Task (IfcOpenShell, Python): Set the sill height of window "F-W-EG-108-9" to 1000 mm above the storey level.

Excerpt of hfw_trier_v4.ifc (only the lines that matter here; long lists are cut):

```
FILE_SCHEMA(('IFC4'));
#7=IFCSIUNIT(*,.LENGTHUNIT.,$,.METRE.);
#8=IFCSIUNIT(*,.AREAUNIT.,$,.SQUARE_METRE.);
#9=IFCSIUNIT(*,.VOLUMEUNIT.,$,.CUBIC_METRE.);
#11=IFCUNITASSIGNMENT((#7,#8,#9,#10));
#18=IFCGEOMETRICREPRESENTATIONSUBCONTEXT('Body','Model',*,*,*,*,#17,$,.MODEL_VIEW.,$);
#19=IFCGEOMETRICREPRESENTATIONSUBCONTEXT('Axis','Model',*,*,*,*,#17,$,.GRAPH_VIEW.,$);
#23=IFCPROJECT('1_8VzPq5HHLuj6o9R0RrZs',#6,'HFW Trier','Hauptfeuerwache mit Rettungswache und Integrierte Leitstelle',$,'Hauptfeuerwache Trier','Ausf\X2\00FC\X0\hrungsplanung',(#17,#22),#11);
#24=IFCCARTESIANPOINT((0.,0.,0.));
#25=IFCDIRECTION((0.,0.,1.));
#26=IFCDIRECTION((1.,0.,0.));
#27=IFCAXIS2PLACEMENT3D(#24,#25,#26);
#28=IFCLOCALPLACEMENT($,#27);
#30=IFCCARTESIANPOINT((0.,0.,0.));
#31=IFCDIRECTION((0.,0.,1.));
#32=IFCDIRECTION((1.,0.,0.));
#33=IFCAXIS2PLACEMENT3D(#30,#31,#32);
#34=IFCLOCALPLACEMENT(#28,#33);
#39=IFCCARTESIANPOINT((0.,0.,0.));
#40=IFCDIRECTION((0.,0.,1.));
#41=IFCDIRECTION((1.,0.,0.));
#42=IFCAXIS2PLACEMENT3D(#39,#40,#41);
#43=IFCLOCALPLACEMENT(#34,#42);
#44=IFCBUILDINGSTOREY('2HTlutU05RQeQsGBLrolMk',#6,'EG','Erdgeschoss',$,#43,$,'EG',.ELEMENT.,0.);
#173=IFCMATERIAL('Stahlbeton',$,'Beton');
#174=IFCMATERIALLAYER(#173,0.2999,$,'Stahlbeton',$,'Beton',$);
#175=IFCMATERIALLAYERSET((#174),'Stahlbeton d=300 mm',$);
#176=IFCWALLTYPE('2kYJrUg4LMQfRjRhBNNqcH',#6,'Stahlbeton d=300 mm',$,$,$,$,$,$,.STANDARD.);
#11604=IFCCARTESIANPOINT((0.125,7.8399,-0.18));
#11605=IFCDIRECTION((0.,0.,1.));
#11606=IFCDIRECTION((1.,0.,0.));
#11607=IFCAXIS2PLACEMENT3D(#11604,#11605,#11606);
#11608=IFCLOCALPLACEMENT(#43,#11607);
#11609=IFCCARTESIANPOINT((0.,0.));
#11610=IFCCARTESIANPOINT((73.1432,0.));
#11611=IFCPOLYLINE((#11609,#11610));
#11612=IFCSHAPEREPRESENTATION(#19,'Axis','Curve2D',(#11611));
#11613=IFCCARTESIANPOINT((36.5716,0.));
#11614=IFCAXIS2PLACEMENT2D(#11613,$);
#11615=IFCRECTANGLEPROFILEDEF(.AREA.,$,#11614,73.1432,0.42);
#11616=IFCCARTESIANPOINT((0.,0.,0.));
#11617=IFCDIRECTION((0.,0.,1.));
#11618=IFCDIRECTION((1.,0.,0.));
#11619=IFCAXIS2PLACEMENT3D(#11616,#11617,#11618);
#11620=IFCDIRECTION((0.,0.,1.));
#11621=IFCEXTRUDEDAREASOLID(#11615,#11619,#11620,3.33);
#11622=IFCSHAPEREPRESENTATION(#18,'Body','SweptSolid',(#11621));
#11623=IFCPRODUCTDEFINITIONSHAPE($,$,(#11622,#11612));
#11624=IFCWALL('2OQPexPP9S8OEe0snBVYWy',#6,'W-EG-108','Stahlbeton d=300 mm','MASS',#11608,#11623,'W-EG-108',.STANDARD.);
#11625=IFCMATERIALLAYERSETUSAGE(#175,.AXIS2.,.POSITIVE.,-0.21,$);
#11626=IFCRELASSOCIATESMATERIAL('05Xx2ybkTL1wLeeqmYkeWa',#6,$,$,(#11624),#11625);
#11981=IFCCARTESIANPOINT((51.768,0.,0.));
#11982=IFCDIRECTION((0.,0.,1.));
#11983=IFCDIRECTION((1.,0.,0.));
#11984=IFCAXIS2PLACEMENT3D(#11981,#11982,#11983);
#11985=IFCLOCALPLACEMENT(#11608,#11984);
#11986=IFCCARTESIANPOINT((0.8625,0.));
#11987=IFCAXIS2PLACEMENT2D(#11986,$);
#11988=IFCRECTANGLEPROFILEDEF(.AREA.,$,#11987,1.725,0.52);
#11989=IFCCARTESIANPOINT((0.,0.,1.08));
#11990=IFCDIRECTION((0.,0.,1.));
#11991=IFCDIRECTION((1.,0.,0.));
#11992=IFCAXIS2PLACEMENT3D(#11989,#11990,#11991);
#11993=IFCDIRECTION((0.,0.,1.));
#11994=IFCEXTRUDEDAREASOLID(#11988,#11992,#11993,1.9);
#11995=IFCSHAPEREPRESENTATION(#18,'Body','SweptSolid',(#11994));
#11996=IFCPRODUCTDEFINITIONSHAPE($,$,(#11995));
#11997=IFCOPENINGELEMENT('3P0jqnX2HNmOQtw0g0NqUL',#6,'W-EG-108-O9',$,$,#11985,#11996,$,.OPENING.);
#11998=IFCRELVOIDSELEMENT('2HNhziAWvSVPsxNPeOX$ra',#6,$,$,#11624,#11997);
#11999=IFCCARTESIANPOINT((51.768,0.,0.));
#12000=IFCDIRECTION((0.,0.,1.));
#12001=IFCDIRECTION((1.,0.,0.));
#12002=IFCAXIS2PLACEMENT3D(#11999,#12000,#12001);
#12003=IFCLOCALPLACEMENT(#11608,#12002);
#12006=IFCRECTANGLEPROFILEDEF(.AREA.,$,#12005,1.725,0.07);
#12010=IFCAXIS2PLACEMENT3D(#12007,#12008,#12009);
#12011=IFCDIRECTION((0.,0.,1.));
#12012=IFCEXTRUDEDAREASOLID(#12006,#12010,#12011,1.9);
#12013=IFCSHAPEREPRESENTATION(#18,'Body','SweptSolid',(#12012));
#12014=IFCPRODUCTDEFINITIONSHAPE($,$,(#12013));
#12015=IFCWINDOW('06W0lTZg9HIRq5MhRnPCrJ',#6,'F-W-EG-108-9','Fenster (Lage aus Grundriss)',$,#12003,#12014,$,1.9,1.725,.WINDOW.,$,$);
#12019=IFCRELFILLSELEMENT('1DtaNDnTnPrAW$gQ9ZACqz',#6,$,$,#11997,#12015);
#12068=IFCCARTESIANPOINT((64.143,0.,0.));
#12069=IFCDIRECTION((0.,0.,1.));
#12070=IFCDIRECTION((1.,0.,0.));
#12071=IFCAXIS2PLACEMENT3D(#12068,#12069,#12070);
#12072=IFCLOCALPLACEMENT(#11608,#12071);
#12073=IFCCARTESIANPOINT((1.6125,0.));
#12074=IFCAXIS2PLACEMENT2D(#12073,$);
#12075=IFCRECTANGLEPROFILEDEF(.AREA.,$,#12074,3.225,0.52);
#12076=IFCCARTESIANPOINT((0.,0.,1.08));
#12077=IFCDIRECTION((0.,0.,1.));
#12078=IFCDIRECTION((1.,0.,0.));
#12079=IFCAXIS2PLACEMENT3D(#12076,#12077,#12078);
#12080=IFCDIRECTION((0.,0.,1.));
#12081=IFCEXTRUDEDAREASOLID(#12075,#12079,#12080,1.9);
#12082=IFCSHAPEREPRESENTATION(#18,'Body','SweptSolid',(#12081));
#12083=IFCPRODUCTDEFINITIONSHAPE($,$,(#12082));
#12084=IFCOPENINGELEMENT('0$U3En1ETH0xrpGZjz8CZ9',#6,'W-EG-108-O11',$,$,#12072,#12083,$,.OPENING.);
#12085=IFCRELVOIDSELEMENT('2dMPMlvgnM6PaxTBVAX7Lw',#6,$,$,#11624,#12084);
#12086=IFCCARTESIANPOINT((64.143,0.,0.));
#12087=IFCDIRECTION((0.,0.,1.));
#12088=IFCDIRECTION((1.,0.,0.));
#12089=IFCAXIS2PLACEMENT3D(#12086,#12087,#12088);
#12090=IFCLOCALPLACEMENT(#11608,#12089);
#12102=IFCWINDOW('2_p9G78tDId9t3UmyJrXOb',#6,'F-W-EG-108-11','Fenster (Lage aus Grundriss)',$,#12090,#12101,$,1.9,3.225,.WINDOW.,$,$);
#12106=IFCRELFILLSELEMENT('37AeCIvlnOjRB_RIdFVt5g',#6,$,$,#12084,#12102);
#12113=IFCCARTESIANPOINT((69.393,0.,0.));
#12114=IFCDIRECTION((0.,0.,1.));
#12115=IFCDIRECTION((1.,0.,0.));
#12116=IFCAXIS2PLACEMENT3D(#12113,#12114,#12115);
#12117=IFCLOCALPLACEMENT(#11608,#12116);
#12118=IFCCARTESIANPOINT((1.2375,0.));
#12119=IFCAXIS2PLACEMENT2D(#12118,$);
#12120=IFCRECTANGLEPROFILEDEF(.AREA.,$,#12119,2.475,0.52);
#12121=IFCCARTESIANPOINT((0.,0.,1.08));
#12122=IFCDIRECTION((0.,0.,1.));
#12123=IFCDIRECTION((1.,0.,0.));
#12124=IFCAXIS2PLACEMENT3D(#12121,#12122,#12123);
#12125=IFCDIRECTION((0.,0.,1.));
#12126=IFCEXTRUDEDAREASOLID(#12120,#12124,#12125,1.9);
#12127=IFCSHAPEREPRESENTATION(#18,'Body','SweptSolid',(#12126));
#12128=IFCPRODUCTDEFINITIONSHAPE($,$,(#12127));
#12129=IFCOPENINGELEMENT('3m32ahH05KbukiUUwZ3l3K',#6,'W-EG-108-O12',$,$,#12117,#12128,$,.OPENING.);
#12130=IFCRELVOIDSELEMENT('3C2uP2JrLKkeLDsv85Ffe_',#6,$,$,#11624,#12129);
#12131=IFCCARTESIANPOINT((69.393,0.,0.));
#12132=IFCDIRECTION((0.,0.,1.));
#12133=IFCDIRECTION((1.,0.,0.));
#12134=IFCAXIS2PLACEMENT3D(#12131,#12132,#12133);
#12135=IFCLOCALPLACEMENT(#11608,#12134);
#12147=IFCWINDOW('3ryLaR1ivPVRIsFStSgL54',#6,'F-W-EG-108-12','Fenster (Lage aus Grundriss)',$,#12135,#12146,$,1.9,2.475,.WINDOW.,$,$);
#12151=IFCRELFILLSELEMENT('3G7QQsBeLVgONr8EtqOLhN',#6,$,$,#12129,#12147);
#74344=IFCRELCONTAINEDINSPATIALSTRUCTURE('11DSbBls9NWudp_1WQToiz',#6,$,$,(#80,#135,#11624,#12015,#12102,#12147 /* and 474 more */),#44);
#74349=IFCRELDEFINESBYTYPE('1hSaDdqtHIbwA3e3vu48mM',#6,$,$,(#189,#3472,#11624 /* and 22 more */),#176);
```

```python
import numpy as np
import ifcopenshell
import ifcopenshell.api.geometry
import ifcopenshell.geom
import ifcopenshell.util.element
import ifcopenshell.util.placement
import ifcopenshell.util.shape
import ifcopenshell.util.unit

model = ifcopenshell.open("hfw_trier_v4.ifc")
unit_scale = ifcopenshell.util.unit.calculate_unit_scale(model)

window = model.by_guid("06W0lTZg9HIRq5MhRnPCrJ")
opening = window.FillsVoids[0].RelatingOpeningElement
storey = ifcopenshell.util.element.get_container(window, ifc_class="IfcBuildingStorey")
level = ifcopenshell.util.placement.get_local_placement(storey.ObjectPlacement)[2, 3]

# The opening's origin need not be at the sill, so measure its lowest point.
shape = ifcopenshell.geom.create_shape(ifcopenshell.geom.settings(), opening)
bottom = ifcopenshell.util.shape.get_shape_bottom_elevation(shape, shape.geometry) / unit_scale
dz = level + 1 / unit_scale - bottom

shift = np.array([0.0, 0.0, dz])
# The window is not placed relative to its opening, so move both.
for product in (opening, window):
    matrix = ifcopenshell.util.placement.get_local_placement(product.ObjectPlacement)
    matrix[:3, 3] += shift
    ifcopenshell.api.geometry.edit_object_placement(model, product=product, matrix=matrix, is_si=False)

print(f"moved by {dz * unit_scale:+.3f} m")

model.write("hfw_trier_v4_updated.ifc")
```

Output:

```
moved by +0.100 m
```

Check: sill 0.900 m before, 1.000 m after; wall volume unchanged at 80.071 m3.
